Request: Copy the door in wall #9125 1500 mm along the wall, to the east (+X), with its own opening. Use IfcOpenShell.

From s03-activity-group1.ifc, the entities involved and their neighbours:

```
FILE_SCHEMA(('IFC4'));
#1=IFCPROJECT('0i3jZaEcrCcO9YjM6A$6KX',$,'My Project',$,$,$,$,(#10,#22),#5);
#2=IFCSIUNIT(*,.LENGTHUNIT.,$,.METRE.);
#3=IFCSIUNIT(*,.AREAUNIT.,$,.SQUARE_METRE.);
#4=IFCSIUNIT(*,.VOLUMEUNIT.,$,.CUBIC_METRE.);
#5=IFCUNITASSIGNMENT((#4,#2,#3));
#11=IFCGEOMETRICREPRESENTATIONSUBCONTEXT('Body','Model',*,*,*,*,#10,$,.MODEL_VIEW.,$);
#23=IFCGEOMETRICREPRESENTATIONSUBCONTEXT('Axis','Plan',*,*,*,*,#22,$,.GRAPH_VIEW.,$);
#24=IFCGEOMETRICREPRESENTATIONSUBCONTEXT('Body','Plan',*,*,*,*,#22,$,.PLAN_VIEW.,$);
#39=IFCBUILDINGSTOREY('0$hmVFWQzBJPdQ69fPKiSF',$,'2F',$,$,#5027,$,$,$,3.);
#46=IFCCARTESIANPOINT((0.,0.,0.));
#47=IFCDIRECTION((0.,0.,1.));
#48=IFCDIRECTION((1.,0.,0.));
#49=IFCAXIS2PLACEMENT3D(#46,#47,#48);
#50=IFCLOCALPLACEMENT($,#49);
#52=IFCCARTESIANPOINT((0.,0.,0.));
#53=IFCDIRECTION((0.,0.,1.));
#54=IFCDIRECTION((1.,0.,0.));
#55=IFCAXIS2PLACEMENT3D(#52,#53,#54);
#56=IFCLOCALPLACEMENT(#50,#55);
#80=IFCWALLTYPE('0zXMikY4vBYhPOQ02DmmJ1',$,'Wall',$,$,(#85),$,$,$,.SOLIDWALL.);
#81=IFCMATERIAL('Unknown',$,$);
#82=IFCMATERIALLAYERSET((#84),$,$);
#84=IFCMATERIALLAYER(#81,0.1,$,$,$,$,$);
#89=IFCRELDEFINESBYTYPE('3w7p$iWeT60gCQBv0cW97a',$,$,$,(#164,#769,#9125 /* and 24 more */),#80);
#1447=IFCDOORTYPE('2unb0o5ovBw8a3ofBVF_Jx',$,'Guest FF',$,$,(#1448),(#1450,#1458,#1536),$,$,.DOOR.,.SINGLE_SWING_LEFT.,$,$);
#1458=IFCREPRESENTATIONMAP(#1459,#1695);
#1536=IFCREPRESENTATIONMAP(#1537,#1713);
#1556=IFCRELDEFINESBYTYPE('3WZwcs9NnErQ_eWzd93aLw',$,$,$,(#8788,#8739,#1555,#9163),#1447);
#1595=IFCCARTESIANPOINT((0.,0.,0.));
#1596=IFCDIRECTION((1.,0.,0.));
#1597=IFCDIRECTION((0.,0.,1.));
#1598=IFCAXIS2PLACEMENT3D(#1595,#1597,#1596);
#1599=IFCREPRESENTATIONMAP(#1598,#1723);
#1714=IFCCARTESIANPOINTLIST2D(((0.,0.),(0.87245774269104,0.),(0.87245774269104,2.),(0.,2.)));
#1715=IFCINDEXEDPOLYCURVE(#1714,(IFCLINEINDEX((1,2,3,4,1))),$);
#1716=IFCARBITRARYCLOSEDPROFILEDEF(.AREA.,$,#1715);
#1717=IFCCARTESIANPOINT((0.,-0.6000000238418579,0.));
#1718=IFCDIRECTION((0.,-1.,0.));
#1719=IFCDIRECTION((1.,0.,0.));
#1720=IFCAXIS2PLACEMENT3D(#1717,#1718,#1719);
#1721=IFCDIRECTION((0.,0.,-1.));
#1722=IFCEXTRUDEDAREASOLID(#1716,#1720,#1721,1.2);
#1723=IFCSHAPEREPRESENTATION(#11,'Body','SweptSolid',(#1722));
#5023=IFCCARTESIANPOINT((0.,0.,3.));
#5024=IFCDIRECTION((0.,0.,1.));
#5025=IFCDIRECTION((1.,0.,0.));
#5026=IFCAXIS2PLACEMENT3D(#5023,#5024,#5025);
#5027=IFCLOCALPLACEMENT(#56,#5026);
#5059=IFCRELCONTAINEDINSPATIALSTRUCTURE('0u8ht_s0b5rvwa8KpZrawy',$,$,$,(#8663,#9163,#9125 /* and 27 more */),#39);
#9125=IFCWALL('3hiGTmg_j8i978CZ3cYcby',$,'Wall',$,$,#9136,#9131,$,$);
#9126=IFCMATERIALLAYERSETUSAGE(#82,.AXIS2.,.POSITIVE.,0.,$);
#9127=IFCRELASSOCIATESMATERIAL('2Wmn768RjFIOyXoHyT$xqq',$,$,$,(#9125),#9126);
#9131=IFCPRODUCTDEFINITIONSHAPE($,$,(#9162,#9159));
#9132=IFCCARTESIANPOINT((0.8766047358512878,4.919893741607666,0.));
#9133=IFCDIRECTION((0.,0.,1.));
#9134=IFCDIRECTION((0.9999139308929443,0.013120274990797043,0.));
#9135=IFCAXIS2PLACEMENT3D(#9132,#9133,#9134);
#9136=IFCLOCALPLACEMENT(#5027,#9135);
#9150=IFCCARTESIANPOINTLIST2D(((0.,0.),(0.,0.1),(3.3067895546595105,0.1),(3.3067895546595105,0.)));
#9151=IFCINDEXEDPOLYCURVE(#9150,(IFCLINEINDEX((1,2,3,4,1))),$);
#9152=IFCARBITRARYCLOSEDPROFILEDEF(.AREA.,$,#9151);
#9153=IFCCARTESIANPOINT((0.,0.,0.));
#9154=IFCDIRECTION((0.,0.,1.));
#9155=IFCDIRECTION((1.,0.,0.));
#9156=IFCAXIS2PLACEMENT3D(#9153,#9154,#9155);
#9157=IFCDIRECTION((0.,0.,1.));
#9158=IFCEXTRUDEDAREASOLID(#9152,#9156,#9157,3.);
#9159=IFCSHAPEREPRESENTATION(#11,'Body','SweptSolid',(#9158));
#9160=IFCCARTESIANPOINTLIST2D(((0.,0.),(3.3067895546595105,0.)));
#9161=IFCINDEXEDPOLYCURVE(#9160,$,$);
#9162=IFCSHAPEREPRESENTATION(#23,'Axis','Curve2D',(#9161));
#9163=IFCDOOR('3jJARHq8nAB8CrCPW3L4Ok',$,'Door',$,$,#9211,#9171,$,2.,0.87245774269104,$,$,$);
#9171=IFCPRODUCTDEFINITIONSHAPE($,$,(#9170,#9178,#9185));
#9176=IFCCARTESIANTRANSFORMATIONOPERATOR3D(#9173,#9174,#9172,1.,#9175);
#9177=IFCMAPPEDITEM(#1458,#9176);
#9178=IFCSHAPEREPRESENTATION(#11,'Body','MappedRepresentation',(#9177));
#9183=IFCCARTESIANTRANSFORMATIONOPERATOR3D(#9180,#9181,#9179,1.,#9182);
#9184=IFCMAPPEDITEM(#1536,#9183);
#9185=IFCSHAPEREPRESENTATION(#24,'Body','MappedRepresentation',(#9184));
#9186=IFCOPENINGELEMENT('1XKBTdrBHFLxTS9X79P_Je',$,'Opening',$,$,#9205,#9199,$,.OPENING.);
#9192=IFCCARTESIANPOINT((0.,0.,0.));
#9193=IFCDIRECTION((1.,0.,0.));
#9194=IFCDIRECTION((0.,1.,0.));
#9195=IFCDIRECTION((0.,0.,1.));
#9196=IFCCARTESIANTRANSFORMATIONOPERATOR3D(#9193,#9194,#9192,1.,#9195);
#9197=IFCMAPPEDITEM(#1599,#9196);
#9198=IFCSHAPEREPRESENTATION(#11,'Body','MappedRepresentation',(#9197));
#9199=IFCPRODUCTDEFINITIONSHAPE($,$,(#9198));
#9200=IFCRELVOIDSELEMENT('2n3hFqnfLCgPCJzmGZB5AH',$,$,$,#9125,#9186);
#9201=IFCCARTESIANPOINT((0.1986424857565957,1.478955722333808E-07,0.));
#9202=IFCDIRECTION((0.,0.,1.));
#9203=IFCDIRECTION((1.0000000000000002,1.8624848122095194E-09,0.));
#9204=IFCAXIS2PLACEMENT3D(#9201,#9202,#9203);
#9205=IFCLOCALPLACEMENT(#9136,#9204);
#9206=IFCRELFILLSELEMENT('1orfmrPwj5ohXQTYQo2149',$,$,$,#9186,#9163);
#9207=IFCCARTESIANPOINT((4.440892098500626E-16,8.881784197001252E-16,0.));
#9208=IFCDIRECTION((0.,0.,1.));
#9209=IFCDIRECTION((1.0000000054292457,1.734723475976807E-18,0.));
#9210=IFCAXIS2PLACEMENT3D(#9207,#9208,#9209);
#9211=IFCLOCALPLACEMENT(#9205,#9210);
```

```python
import ifcopenshell
import ifcopenshell.api.feature
import ifcopenshell.api.geometry
import ifcopenshell.api.root
import ifcopenshell.geom
import ifcopenshell.util.element
import ifcopenshell.util.placement
import ifcopenshell.util.shape
import ifcopenshell.util.unit

model = ifcopenshell.open("s03-activity-group1.ifc")
unit_scale = ifcopenshell.util.unit.calculate_unit_scale(model)
settings = ifcopenshell.geom.settings()


def volume(element):
    """Net volume in cubic metres, openings subtracted."""
    shape = ifcopenshell.geom.create_shape(settings, element)
    return ifcopenshell.util.shape.get_volume(shape.geometry)


door = model.by_guid("3jJARHq8nAB8CrCPW3L4Ok")
opening = door.FillsVoids[0].RelatingOpeningElement
wall = opening.VoidsElements[0].RelatingBuildingElement
before = volume(wall)
shift = ifcopenshell.util.placement.get_local_placement(wall.ObjectPlacement)[:3, 0] * 1.5 / unit_scale

# copy_class copies the void relationship, type, container and properties, but no geometry.
new_opening = ifcopenshell.api.root.copy_class(model, product=opening)
new_opening.Representation = ifcopenshell.util.element.copy_deep(
    model, opening.Representation, exclude=["IfcGeometricRepresentationContext", "IfcRepresentationMap"]
)
new_door = ifcopenshell.api.root.copy_class(model, product=door)
new_door.Representation = ifcopenshell.util.element.copy_deep(
    model, door.Representation, exclude=["IfcGeometricRepresentationContext", "IfcRepresentationMap"]
)
ifcopenshell.api.feature.add_filling(model, opening=new_opening, element=new_door)

for old, new in ((opening, new_opening), (door, new_door)):
    matrix = ifcopenshell.util.placement.get_local_placement(old.ObjectPlacement)
    matrix[:3, 3] += shift
    ifcopenshell.api.geometry.edit_object_placement(model, product=new, matrix=matrix, is_si=False)

after = volume(wall)

print(f"wall volume {before:.3f} -> {after:.3f} m3")

model.write("s03-activity-group1_v2.ifc")
```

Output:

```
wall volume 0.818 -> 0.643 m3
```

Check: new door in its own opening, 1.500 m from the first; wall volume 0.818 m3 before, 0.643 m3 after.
